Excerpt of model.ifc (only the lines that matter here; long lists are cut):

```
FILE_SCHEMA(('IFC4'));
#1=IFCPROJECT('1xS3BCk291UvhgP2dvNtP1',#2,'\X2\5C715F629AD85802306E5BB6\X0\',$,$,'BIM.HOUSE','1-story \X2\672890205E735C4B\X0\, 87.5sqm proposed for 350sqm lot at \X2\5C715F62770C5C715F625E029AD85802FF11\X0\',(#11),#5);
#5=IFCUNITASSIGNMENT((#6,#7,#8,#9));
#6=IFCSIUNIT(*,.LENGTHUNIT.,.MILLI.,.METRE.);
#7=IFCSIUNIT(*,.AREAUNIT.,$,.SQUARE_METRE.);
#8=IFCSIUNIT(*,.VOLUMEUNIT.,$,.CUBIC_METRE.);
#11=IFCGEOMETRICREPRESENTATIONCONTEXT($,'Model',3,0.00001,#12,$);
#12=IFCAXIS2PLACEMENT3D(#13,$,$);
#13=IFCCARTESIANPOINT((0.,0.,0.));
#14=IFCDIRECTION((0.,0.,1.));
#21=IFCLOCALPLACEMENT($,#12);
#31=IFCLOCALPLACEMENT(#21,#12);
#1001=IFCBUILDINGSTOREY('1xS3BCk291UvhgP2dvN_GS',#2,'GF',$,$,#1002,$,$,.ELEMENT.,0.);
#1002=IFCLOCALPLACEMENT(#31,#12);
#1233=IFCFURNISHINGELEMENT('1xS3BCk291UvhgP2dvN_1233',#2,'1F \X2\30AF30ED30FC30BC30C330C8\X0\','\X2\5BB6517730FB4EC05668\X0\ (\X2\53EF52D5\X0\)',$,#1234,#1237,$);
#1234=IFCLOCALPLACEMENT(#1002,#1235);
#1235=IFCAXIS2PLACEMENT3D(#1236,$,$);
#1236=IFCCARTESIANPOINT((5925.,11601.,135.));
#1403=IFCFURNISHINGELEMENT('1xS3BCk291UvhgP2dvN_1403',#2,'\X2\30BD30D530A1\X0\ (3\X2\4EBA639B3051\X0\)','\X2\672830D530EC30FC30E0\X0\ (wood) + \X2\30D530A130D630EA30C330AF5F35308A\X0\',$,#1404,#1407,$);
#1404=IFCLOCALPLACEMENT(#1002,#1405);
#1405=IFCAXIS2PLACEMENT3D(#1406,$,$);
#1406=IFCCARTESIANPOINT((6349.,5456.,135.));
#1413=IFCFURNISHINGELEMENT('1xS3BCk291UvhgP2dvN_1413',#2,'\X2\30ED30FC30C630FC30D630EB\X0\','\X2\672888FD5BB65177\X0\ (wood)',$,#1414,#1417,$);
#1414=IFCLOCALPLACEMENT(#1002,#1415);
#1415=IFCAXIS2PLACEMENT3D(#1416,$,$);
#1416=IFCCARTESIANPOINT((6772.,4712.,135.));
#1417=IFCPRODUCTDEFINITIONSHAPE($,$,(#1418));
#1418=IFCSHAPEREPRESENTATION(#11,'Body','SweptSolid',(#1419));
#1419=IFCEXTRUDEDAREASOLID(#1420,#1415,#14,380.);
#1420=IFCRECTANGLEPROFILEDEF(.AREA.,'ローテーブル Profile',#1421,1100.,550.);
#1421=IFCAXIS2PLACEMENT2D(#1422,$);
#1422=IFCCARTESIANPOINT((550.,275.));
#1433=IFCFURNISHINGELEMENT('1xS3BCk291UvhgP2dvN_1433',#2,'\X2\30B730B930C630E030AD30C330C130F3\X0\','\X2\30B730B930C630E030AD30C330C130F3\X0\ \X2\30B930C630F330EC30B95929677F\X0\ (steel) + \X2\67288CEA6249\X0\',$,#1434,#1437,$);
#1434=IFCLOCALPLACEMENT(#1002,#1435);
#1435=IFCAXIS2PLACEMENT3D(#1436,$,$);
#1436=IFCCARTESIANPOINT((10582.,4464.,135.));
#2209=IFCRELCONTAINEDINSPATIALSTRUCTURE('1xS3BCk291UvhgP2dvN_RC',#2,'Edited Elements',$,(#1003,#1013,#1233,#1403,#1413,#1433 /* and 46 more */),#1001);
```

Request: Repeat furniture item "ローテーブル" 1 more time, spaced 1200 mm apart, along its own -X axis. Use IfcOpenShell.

```python
import ifcopenshell
import ifcopenshell.api.geometry
import ifcopenshell.api.root
import ifcopenshell.util.element
import ifcopenshell.util.placement

model = ifcopenshell.open("model.ifc")


def reuse_history(source, copy):
    """copy_class also copies each property set's owner history, people and application; keep the originals."""
    for rel in copy.IsDefinedBy:
        if rel.is_a("IfcRelDefinesByProperties") and (history := rel.RelatingPropertyDefinition.OwnerHistory):
            rel.RelatingPropertyDefinition.OwnerHistory = source.OwnerHistory
            ifcopenshell.util.element.remove_deep2(model, history)


source = model.by_id(1413)
base = ifcopenshell.util.placement.get_local_placement(source.ObjectPlacement)
step = -base[:3, 0] * 1200.0

for i in range(1, 2):
    copy = ifcopenshell.api.root.copy_class(model, product=source)
    copy.Representation = ifcopenshell.util.element.copy_deep(
        model, source.Representation, exclude=["IfcGeometricRepresentationContext", "IfcRepresentationMap"]
    )
    reuse_history(source, copy)
    matrix = base.copy()
    matrix[:3, 3] += i * step
    print("added at", matrix[:3, 3].round(3) + 0.0)
    ifcopenshell.api.geometry.edit_object_placement(model, product=copy, matrix=matrix, is_si=False)

model.write("model_rev.ifc")
```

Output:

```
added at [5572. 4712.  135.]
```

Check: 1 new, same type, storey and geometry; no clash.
